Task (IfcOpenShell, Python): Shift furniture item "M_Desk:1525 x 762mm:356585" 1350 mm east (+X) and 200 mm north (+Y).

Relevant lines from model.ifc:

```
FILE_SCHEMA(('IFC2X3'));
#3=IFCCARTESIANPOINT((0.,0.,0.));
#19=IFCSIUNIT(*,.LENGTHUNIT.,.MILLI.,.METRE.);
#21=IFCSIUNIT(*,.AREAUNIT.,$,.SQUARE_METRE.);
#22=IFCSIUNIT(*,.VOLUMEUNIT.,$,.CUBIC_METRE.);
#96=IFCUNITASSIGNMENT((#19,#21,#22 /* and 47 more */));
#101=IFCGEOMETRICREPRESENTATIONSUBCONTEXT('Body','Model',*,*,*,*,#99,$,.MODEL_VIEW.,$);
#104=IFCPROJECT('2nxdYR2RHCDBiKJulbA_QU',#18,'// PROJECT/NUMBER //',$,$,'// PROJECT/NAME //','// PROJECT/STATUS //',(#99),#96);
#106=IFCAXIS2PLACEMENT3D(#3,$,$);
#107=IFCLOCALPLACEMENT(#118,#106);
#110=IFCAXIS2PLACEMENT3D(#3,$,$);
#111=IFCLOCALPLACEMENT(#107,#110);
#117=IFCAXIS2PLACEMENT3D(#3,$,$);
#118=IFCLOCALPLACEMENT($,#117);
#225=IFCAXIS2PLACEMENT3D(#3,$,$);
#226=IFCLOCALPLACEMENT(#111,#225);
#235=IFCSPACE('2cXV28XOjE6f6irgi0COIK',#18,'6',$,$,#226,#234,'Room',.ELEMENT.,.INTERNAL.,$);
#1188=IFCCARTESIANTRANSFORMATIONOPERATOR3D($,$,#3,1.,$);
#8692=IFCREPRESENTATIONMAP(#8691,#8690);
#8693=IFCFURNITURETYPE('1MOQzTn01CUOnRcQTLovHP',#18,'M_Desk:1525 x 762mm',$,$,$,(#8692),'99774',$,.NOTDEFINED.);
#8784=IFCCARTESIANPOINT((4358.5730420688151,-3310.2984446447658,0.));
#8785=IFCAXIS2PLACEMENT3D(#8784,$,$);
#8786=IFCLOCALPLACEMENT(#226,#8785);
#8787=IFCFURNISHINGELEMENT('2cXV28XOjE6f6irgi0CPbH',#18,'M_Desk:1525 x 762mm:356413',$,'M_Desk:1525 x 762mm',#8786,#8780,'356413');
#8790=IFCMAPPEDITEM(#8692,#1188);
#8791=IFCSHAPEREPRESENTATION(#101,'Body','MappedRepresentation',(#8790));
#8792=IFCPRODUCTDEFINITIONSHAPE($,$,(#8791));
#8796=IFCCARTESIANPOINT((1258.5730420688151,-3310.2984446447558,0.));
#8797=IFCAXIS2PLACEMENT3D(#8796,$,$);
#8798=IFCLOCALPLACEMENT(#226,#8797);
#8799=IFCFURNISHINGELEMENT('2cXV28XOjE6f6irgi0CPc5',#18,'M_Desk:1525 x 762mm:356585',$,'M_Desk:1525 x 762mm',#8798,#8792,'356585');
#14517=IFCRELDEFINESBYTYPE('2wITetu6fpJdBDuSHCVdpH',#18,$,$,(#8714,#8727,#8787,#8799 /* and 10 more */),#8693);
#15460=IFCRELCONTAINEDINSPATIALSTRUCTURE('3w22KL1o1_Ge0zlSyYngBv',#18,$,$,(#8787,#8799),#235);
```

```python
import ifcopenshell
import ifcopenshell.api.geometry
import ifcopenshell.util.placement
import ifcopenshell.util.unit

model = ifcopenshell.open("model.ifc")
unit_scale = ifcopenshell.util.unit.calculate_unit_scale(model)

item = model.by_guid("2cXV28XOjE6f6irgi0CPc5")
matrix = ifcopenshell.util.placement.get_local_placement(item.ObjectPlacement)
matrix[0, 3] += 1.35 / unit_scale
matrix[1, 3] += 0.2 / unit_scale
ifcopenshell.api.geometry.edit_object_placement(model, product=item, matrix=matrix, is_si=False)

print(ifcopenshell.util.placement.get_local_placement(item.ObjectPlacement).round(3) + 0.0)

model.write("model-out.ifc")
```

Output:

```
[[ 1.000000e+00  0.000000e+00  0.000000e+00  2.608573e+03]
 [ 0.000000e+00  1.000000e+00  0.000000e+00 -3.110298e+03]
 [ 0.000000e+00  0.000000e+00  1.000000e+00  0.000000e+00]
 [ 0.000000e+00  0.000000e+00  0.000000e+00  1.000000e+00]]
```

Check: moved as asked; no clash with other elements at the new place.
